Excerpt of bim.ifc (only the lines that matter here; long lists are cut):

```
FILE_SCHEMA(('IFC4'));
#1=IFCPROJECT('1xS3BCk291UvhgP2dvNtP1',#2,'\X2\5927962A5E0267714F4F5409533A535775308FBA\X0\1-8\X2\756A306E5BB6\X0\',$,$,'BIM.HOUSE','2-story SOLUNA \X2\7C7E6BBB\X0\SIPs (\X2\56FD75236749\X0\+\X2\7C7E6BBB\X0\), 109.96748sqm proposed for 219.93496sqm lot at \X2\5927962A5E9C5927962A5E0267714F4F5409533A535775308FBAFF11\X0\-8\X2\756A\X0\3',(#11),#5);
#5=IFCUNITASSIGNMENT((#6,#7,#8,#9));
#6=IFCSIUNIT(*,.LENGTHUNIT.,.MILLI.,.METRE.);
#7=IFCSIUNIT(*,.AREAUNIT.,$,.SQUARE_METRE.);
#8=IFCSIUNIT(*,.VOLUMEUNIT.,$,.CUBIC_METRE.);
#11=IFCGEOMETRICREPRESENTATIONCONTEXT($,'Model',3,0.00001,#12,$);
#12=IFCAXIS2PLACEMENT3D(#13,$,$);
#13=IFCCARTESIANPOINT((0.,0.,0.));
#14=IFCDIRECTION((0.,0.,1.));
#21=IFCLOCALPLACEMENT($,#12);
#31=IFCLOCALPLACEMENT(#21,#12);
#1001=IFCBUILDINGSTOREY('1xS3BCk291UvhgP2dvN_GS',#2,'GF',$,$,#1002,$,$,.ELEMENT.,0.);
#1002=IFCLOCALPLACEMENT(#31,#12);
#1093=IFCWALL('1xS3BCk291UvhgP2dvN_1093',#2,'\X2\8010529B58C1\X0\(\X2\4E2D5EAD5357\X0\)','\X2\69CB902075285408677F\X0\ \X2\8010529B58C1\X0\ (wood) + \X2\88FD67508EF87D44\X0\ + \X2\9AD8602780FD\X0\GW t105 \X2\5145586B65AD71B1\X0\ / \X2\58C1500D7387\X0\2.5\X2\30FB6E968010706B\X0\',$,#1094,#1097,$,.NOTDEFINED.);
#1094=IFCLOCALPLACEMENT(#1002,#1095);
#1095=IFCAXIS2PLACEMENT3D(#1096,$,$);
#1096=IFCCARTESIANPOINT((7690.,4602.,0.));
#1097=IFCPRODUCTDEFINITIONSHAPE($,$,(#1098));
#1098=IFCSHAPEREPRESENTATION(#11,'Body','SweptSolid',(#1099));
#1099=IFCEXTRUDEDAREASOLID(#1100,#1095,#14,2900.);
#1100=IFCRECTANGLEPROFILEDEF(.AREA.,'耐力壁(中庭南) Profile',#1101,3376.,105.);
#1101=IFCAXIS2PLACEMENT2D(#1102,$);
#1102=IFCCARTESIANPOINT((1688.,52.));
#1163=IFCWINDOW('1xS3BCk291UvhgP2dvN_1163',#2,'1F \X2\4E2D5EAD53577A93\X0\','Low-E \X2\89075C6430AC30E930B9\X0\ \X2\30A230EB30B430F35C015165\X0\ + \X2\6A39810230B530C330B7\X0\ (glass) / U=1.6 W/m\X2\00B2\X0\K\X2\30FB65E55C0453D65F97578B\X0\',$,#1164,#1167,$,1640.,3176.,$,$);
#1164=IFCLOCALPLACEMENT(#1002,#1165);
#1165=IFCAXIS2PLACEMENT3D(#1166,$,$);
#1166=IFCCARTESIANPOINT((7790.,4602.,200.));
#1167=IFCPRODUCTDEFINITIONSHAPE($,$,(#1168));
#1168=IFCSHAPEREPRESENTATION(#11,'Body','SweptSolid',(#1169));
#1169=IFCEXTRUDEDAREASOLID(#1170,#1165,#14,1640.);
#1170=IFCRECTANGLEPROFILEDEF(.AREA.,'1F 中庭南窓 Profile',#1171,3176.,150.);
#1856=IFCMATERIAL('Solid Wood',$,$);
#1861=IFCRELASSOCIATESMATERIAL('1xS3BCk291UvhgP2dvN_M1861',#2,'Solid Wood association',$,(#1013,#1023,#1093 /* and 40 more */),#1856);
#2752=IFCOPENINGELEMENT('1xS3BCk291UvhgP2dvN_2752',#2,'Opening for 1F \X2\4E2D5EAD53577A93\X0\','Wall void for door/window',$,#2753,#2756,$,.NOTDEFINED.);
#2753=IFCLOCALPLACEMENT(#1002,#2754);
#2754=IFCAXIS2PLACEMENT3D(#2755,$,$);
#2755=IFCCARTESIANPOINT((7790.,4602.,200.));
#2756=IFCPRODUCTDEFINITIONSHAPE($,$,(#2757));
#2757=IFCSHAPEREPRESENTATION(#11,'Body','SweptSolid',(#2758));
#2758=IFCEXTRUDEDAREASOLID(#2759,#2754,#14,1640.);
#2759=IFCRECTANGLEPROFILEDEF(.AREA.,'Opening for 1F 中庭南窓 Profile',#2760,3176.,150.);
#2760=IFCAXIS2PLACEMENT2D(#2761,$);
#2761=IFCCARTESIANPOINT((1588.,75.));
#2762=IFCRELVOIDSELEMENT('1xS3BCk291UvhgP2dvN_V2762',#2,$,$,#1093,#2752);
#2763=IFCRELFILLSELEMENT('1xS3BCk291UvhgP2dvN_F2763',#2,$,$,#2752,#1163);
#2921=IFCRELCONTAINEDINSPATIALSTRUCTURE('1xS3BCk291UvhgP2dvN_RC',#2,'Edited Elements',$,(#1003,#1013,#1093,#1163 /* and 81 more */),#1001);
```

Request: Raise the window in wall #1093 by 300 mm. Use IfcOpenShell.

```python
import numpy as np
import ifcopenshell
import ifcopenshell.api.geometry
import ifcopenshell.util.placement
import ifcopenshell.util.unit

model = ifcopenshell.open("bim.ifc")
unit_scale = ifcopenshell.util.unit.calculate_unit_scale(model)

window = model.by_id(1163)
opening = window.FillsVoids[0].RelatingOpeningElement
dz = 0.3 / unit_scale

shift = np.array([0.0, 0.0, dz])
# The window is not placed relative to its opening, so move both.
for product in (opening, window):
    matrix = ifcopenshell.util.placement.get_local_placement(product.ObjectPlacement)
    matrix[:3, 3] += shift
    ifcopenshell.api.geometry.edit_object_placement(model, product=product, matrix=matrix, is_si=False)

print(f"moved by {dz * unit_scale:+.3f} m")

model.write("bim_v2.ifc")
```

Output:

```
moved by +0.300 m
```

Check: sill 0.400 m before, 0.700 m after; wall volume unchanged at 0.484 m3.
